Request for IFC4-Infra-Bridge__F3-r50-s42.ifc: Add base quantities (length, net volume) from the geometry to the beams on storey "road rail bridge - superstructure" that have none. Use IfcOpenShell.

First a look at what the model holds.

```python
import ifcopenshell
import ifcopenshell.util.element
import ifcopenshell.util.unit

model = ifcopenshell.open("IFC4-Infra-Bridge__F3-r50-s42.ifc")
print(model.schema)
for unit_type in ("LENGTHUNIT", "AREAUNIT", "VOLUMEUNIT"):
    print(unit_type, ifcopenshell.util.unit.calculate_unit_scale(model, unit_type))
storey = next(s for s in model.by_type("IfcBuildingStorey") if s.Name == "road rail bridge - superstructure")
beams = [e for e in ifcopenshell.util.element.get_decomposition(storey) if e.is_a("IfcBeam")]
for e in sorted(beams, key=lambda e: e.id()):
    print(e.id(), e.is_a(), e.Name, list(ifcopenshell.util.element.get_psets(e, qtos_only=True)), sep=" | ")
```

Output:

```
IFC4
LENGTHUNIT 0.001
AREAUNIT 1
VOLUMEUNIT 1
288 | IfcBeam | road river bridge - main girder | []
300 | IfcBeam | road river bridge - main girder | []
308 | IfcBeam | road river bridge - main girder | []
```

```python
import ifcopenshell
import ifcopenshell.api.pset
import ifcopenshell.geom
import ifcopenshell.util.element
import ifcopenshell.util.shape
import ifcopenshell.util.unit

model = ifcopenshell.open("IFC4-Infra-Bridge__F3-r50-s42.ifc")
unit_scale = ifcopenshell.util.unit.calculate_unit_scale(model)
volume_scale = ifcopenshell.util.unit.calculate_unit_scale(model, "VOLUMEUNIT")
settings = ifcopenshell.geom.settings()

storey = next(s for s in model.by_type("IfcBuildingStorey") if s.Name == "road rail bridge - superstructure")
beams = [e for e in ifcopenshell.util.element.get_decomposition(storey) if e.is_a("IfcBeam")]

for e in sorted(beams, key=lambda e: e.id()):
    if ifcopenshell.util.element.get_psets(e, qtos_only=True, should_inherit=False):
        continue
    # Geometry comes back in metres, in the element's own axes.
    shape = ifcopenshell.geom.create_shape(settings, e)
    values = {
        "Length": ifcopenshell.util.shape.get_max_xyz(shape.geometry) / unit_scale,
        "NetVolume": ifcopenshell.util.shape.get_volume(shape.geometry) / volume_scale,
    }
    qto = ifcopenshell.api.pset.add_qto(model, product=e, name="Qto_BeamBaseQuantities")
    ifcopenshell.api.pset.edit_qto(model, qto=qto, properties=values)
    print(e.id(), {k: round(v, 3) for k, v in values.items()})

model.write("IFC4-Infra-Bridge__F3-r50-s42_updated.ifc")
```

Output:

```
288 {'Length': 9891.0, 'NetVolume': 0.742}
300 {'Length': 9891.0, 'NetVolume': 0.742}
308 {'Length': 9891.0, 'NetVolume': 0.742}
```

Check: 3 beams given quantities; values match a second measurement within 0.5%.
